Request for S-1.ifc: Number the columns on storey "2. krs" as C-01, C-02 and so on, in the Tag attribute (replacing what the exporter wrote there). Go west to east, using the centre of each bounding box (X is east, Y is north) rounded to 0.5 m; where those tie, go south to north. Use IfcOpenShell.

First a look at what the model holds.

```python
import ifcopenshell
import ifcopenshell.util.element
import ifcopenshell.util.placement

model = ifcopenshell.open("S-1.ifc")
print(model.schema)
storey = next(s for s in model.by_type("IfcBuildingStorey") if s.Name == "2. krs")
columns = [e for e in ifcopenshell.util.element.get_decomposition(storey) if e.is_a("IfcColumn")]
for e in sorted(columns, key=lambda e: e.id()):
    origin = ifcopenshell.util.placement.get_local_placement(e.ObjectPlacement)[:3, 3]
    print(e.id(), e.Tag, e.Name, origin.round(2) + 0.0, sep=" | ")
```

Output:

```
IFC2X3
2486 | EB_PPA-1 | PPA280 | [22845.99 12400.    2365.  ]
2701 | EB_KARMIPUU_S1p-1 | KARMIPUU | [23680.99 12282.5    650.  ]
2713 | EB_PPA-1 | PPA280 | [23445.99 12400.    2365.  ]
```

```python
import ifcopenshell
import ifcopenshell.geom
import ifcopenshell.util.element
import ifcopenshell.util.shape

model = ifcopenshell.open("S-1.ifc")
settings = ifcopenshell.geom.settings()
settings.set("use-world-coords", True)


def centre(element):
    shape = ifcopenshell.geom.create_shape(settings, element)
    return ifcopenshell.util.shape.get_bbox_centroid(shape.geometry)


storey = next(s for s in model.by_type("IfcBuildingStorey") if s.Name == "2. krs")
columns = [e for e in ifcopenshell.util.element.get_decomposition(storey) if e.is_a("IfcColumn")]

# Insertion points can sit at a corner or the storey origin, so sort by the geometry (in metres).
centres = {e: centre(e) for e in columns}
columns.sort(key=lambda e: (round(centres[e][0] / 0.5), centres[e][1]))

for i, e in enumerate(columns, start=1):
    number = f"C-{i:02d}"
    e.Tag = number
    print(e.id(), number)

model.write("S-1_edited.ifc")
```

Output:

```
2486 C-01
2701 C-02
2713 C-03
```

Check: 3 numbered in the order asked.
